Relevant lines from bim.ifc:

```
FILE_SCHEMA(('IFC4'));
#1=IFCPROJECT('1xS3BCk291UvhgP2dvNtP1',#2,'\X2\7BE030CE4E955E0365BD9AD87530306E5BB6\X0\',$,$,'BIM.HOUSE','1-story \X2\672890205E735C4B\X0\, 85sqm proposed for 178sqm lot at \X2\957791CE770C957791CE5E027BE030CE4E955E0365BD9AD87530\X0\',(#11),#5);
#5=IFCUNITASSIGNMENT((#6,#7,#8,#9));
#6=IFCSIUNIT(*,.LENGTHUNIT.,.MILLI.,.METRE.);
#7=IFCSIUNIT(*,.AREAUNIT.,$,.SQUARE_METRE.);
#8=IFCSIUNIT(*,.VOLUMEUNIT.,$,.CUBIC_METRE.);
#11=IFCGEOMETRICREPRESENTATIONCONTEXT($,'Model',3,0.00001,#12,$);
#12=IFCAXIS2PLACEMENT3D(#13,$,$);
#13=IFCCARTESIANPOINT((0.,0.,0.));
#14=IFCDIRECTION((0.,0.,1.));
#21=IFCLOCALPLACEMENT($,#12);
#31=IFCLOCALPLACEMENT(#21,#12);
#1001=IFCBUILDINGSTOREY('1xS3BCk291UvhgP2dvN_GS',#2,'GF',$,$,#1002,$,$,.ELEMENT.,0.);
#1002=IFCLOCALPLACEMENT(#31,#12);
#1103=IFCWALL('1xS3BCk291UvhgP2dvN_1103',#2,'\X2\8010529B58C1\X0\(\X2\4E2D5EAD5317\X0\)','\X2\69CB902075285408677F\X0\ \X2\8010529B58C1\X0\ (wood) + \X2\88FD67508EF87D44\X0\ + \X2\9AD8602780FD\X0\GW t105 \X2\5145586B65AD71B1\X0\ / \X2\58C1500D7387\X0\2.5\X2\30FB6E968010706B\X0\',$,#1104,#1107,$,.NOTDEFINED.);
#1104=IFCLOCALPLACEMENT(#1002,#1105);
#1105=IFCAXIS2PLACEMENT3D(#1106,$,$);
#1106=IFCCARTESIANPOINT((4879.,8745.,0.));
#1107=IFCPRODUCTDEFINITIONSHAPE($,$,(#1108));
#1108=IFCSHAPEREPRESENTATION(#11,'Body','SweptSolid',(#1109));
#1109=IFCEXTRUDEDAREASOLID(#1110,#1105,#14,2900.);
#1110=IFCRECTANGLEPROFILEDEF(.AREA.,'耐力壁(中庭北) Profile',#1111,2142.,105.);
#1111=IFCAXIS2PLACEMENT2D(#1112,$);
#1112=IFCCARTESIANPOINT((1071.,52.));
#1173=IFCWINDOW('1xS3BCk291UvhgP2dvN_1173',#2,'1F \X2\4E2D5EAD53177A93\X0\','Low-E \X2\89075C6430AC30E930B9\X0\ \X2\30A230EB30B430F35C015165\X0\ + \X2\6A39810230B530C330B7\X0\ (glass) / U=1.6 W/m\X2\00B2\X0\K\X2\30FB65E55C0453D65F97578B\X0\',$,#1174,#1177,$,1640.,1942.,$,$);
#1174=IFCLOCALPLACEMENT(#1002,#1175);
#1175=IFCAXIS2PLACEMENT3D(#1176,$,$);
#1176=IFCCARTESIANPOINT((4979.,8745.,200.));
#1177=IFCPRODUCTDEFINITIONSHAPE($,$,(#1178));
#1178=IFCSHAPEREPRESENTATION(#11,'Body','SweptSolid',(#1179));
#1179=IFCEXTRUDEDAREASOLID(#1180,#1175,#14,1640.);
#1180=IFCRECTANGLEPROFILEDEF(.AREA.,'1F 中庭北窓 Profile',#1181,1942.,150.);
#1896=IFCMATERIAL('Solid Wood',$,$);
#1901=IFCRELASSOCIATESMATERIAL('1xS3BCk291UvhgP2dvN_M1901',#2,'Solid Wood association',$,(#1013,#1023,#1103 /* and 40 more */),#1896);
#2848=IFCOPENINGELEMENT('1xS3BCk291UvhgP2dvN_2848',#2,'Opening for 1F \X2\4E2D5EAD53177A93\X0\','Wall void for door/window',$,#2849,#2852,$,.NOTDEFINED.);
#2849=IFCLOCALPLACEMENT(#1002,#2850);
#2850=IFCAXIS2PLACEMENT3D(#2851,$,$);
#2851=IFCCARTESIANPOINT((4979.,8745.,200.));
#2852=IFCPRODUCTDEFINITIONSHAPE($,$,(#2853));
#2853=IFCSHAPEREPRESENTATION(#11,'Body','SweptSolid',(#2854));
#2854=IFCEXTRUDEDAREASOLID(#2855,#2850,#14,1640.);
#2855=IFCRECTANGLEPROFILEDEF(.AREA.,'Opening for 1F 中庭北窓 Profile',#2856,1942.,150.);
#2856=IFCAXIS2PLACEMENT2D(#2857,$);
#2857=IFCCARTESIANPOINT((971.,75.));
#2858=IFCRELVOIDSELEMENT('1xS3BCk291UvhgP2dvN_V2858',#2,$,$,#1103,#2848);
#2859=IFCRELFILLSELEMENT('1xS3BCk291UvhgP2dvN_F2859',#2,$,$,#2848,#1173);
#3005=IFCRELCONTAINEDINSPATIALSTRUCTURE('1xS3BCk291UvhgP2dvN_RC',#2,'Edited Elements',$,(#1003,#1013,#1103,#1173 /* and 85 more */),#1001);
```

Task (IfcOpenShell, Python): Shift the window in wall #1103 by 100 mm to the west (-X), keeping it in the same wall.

```python
import ifcopenshell
import ifcopenshell.api.geometry
import ifcopenshell.util.placement
import ifcopenshell.util.unit

model = ifcopenshell.open("bim.ifc")
unit_scale = ifcopenshell.util.unit.calculate_unit_scale(model)

window = model.by_guid("1xS3BCk291UvhgP2dvN_1173")
opening = window.FillsVoids[0].RelatingOpeningElement
wall = opening.VoidsElements[0].RelatingBuildingElement

wall_matrix = ifcopenshell.util.placement.get_local_placement(wall.ObjectPlacement)
shift = wall_matrix[:3, 0] * -0.1 / unit_scale
before = ifcopenshell.util.placement.get_local_placement(window.ObjectPlacement)[:3, 3].copy()

# The window is not placed relative to its opening, so move both.
for product in (opening, window):
    matrix = ifcopenshell.util.placement.get_local_placement(product.ObjectPlacement)
    matrix[:3, 3] += shift
    ifcopenshell.api.geometry.edit_object_placement(model, product=product, matrix=matrix, is_si=False)

after = ifcopenshell.util.placement.get_local_placement(window.ObjectPlacement)[:3, 3]
print("window moved by", (after - before).round(3) + 0.0)

model.write("bim_updated.ifc")
```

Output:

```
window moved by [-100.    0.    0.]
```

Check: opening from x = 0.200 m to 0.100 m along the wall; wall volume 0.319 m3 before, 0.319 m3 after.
